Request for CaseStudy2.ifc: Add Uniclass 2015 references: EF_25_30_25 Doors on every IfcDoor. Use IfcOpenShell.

First a look at what the model holds.

```python
import ifcopenshell

model = ifcopenshell.open("CaseStudy2.ifc")
print(model.schema)
print("classifications:", [c.Name for c in model.by_type("IfcClassification")])
for ifc_class in ("IfcDoor", "IfcRoof", "IfcStair", "IfcWall", "IfcWindow"):
    print(ifc_class, len(model.by_type(ifc_class)))
```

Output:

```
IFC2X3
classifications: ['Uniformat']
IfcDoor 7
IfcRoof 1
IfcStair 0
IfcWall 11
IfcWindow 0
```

```python
import ifcopenshell
import ifcopenshell.api.classification

model = ifcopenshell.open("CaseStudy2.ifc")

# IFC2X3 requires Source and Edition and has no link from the project to the system.
system = model.create_entity("IfcClassification", Source="NBS", Edition="2015", Name="Uniclass 2015")

codes = {
    "IfcDoor": ("EF_25_30_25", "Doors"),
}
for ifc_class, (code, name) in codes.items():
    products = model.by_type(ifc_class)
    ifcopenshell.api.classification.add_reference(
        model, products=products, classification=system, identification=code, name=name
    )
    print(code, len(products))

model.write("CaseStudy2_v2.ifc")
```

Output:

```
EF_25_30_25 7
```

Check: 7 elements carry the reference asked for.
